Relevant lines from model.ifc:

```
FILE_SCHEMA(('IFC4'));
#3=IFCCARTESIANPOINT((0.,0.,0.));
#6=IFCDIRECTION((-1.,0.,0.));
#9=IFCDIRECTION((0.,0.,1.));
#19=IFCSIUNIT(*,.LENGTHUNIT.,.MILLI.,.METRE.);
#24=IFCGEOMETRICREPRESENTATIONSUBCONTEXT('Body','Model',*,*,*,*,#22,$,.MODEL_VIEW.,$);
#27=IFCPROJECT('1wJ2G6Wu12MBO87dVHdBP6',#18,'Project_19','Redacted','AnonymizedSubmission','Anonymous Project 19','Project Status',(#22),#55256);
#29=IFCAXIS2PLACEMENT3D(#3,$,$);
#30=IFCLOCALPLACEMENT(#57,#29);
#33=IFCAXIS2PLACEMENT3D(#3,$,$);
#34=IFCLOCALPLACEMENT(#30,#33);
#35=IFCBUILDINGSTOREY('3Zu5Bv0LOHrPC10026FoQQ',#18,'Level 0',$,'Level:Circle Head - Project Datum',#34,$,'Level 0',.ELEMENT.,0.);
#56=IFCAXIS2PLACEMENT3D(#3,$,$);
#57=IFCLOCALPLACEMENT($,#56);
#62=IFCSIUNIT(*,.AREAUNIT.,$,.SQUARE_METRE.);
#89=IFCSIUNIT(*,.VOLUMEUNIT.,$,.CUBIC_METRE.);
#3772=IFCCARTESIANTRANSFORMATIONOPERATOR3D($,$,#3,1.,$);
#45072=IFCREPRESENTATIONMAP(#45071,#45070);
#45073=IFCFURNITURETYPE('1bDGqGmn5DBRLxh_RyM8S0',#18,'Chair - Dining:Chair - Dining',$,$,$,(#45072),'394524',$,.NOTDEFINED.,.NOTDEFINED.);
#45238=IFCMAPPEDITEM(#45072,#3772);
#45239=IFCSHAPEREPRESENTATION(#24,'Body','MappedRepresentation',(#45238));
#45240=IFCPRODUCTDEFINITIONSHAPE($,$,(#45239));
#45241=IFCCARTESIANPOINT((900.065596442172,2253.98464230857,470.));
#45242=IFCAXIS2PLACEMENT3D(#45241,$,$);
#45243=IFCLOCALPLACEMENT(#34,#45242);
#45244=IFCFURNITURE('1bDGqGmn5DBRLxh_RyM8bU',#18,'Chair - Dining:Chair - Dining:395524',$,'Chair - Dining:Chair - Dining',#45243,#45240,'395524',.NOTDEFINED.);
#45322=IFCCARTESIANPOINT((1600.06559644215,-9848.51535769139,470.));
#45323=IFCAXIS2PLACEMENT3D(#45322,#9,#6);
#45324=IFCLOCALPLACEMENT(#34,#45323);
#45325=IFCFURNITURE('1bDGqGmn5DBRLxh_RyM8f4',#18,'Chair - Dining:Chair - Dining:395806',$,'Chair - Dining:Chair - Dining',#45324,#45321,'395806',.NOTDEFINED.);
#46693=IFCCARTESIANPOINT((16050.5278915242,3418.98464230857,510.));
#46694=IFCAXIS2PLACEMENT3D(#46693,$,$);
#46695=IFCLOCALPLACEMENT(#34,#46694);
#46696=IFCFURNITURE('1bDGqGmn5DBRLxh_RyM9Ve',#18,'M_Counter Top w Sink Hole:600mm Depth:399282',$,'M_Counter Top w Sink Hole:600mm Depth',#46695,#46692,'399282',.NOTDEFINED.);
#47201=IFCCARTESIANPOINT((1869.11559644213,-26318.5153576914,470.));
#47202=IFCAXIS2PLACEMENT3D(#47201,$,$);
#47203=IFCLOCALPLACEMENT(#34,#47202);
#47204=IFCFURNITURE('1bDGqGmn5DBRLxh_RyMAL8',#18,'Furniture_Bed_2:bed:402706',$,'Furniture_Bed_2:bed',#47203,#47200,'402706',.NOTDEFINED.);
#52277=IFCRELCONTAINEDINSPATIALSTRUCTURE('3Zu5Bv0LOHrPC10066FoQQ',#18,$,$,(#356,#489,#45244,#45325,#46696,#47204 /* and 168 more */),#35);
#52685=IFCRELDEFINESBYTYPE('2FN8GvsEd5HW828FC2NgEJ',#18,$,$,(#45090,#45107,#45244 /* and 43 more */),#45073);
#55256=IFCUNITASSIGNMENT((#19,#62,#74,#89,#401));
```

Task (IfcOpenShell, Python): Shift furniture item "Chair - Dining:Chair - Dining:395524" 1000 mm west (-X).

```python
import ifcopenshell
import ifcopenshell.api.geometry
import ifcopenshell.util.placement

model = ifcopenshell.open("model.ifc")

item = model.by_guid("1bDGqGmn5DBRLxh_RyM8bU")
matrix = ifcopenshell.util.placement.get_local_placement(item.ObjectPlacement)
matrix[0, 3] -= 1000.0
ifcopenshell.api.geometry.edit_object_placement(model, product=item, matrix=matrix, is_si=False)

print(ifcopenshell.util.placement.get_local_placement(item.ObjectPlacement).round(3) + 0.0)

model.write("model_v2.ifc")
```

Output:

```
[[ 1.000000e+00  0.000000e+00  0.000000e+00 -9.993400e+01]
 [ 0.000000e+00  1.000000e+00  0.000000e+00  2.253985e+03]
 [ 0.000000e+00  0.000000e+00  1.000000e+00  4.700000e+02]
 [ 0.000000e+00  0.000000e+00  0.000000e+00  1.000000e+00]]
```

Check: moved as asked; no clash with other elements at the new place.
